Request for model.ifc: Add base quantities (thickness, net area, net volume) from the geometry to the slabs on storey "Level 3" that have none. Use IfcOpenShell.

First a look at what the model holds.

```python
import ifcopenshell
import ifcopenshell.util.element
import ifcopenshell.util.unit

model = ifcopenshell.open("model.ifc")
print(model.schema)
for unit_type in ("LENGTHUNIT", "AREAUNIT", "VOLUMEUNIT"):
    print(unit_type, ifcopenshell.util.unit.calculate_unit_scale(model, unit_type))
storey = next(s for s in model.by_type("IfcBuildingStorey") if s.Name == "Level 3")
slabs = [e for e in ifcopenshell.util.element.get_decomposition(storey) if e.is_a("IfcSlab")]
for e in sorted(slabs, key=lambda e: e.id()):
    print(e.id(), e.is_a(), e.Name, list(ifcopenshell.util.element.get_psets(e, qtos_only=True)), sep=" | ")
```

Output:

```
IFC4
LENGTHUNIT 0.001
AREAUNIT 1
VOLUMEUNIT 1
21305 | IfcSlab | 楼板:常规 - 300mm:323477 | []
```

```python
import ifcopenshell
import ifcopenshell.api.pset
import ifcopenshell.geom
import ifcopenshell.util.element
import ifcopenshell.util.shape
import ifcopenshell.util.unit

model = ifcopenshell.open("model.ifc")
unit_scale = ifcopenshell.util.unit.calculate_unit_scale(model)
area_scale = ifcopenshell.util.unit.calculate_unit_scale(model, "AREAUNIT")
volume_scale = ifcopenshell.util.unit.calculate_unit_scale(model, "VOLUMEUNIT")
settings = ifcopenshell.geom.settings()

storey = next(s for s in model.by_type("IfcBuildingStorey") if s.Name == "Level 3")
slabs = [e for e in ifcopenshell.util.element.get_decomposition(storey) if e.is_a("IfcSlab")]

for e in sorted(slabs, key=lambda e: e.id()):
    if ifcopenshell.util.element.get_psets(e, qtos_only=True, should_inherit=False):
        continue
    # Geometry comes back in metres, in the element's own axes.
    shape = ifcopenshell.geom.create_shape(settings, e)
    values = {
        "Width": ifcopenshell.util.shape.get_z(shape.geometry) / unit_scale,
        "NetArea": ifcopenshell.util.shape.get_footprint_area(shape.geometry) / area_scale,
        "NetVolume": ifcopenshell.util.shape.get_volume(shape.geometry) / volume_scale,
    }
    qto = ifcopenshell.api.pset.add_qto(model, product=e, name="Qto_SlabBaseQuantities")
    ifcopenshell.api.pset.edit_qto(model, qto=qto, properties=values)
    print(e.id(), {k: round(v, 3) for k, v in values.items()})

model.write("model-out.ifc")
```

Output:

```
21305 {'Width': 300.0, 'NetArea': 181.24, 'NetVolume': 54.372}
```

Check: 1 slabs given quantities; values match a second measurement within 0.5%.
